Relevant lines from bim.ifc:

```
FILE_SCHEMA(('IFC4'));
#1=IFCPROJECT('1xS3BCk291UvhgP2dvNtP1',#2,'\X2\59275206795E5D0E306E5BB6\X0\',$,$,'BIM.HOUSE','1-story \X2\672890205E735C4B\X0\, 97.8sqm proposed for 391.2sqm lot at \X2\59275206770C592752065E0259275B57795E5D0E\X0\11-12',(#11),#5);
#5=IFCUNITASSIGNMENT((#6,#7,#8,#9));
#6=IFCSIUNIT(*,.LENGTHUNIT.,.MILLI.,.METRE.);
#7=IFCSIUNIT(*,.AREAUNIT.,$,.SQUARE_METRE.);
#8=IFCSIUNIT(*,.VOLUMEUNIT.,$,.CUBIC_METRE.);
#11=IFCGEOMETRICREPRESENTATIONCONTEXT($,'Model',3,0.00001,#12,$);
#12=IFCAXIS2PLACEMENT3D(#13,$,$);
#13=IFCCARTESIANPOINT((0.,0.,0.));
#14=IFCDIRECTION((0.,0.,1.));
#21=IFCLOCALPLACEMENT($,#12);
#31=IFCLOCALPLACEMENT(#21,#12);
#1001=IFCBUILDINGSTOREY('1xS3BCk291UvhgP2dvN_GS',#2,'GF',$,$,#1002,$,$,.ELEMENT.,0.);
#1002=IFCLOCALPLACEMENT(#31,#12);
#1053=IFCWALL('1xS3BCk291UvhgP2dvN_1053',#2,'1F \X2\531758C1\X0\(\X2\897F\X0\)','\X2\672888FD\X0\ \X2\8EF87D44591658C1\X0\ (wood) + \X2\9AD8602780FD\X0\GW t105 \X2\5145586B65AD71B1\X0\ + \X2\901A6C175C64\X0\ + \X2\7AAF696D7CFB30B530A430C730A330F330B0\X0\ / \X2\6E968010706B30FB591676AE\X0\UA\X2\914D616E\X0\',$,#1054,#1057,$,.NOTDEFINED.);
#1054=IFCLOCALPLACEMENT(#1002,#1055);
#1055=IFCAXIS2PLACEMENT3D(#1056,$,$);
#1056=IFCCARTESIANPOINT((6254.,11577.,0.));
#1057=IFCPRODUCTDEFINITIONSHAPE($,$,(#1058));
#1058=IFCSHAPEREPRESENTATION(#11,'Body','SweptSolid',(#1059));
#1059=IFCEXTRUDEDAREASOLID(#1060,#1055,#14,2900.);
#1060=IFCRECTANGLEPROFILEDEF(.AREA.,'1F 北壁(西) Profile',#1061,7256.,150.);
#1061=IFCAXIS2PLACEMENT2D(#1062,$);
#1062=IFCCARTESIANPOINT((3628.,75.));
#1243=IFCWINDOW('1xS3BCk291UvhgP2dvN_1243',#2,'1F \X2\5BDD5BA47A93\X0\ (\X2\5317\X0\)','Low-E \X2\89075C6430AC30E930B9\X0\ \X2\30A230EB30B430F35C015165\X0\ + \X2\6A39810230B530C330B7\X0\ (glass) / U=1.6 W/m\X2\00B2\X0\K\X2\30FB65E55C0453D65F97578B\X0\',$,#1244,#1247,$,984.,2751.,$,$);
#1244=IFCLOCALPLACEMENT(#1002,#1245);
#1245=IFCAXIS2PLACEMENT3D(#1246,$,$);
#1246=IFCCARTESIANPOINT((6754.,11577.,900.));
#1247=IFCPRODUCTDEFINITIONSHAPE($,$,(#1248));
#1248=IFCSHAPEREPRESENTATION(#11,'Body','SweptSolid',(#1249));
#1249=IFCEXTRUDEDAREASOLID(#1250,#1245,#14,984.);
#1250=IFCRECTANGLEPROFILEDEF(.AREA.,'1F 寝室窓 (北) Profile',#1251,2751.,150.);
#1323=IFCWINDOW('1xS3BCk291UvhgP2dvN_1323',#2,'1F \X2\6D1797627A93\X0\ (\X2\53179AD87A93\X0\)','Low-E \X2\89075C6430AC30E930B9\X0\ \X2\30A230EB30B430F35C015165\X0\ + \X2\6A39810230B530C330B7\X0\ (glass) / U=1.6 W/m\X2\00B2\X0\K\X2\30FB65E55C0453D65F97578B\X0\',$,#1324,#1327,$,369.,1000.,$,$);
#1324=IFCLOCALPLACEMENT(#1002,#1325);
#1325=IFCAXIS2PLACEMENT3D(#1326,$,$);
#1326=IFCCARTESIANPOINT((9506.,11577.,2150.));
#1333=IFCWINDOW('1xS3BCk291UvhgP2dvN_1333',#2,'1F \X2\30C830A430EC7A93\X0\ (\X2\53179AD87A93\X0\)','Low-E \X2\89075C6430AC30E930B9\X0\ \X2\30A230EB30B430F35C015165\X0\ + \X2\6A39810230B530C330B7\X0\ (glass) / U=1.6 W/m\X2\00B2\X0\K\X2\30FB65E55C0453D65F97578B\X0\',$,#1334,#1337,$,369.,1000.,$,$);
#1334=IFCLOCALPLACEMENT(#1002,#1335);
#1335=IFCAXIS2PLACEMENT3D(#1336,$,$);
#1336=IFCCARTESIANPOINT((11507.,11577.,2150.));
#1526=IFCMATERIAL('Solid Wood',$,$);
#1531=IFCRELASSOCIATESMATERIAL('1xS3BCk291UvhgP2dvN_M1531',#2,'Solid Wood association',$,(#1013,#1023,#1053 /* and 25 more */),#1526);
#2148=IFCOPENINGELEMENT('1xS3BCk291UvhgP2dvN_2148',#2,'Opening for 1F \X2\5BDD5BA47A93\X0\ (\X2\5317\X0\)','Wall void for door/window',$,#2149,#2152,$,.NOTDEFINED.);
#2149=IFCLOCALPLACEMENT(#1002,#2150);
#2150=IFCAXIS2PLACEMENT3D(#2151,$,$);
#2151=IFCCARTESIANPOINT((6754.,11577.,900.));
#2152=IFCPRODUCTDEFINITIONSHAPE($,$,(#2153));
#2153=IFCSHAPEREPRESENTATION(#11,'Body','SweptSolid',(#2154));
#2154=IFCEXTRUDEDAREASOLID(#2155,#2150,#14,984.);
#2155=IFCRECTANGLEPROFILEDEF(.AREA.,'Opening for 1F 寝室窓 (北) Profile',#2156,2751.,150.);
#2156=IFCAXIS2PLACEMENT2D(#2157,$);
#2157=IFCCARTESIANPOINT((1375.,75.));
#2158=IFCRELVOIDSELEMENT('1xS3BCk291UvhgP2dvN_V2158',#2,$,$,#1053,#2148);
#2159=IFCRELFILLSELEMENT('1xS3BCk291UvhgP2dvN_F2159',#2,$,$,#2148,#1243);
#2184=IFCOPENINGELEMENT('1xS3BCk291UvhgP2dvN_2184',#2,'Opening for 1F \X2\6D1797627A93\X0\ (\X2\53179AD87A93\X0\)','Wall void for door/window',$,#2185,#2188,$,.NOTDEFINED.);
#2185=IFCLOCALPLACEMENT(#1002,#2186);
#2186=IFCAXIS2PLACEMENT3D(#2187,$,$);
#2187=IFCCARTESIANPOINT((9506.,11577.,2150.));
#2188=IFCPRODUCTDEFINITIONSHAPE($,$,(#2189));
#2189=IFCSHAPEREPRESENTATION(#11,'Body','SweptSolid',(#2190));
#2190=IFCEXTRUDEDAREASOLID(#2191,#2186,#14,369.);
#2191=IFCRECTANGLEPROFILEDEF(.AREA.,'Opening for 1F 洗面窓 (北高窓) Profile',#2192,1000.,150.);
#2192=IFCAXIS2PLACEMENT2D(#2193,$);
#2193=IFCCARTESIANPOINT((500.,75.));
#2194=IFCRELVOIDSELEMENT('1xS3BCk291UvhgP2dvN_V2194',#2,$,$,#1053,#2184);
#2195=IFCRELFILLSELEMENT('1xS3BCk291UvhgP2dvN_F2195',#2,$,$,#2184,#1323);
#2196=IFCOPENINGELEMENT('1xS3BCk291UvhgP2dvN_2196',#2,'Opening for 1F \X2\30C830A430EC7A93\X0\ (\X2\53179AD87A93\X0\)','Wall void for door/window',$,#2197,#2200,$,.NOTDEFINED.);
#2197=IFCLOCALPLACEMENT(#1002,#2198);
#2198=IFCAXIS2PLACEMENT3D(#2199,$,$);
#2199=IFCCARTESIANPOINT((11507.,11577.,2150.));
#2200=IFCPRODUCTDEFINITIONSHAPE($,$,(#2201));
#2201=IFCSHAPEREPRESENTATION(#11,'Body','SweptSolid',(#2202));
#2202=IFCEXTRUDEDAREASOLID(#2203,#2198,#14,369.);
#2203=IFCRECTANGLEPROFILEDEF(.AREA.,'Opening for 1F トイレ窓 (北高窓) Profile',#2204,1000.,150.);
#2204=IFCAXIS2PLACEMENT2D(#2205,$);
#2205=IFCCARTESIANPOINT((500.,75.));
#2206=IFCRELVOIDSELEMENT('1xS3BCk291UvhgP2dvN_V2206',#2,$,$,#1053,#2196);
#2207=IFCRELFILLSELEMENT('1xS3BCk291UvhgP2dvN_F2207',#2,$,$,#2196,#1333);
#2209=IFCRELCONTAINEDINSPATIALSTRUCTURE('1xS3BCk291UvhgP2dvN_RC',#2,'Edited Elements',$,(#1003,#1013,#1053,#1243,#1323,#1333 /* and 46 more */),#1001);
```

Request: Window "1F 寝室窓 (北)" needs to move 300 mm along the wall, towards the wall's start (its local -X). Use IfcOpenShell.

```python
import ifcopenshell
import ifcopenshell.api.geometry
import ifcopenshell.util.placement

model = ifcopenshell.open("bim.ifc")

window = model.by_guid("1xS3BCk291UvhgP2dvN_1243")
opening = window.FillsVoids[0].RelatingOpeningElement
wall = opening.VoidsElements[0].RelatingBuildingElement

wall_matrix = ifcopenshell.util.placement.get_local_placement(wall.ObjectPlacement)
shift = wall_matrix[:3, 0] * -300.0
before = ifcopenshell.util.placement.get_local_placement(window.ObjectPlacement)[:3, 3].copy()

# The window is not placed relative to its opening, so move both.
for product in (opening, window):
    matrix = ifcopenshell.util.placement.get_local_placement(product.ObjectPlacement)
    matrix[:3, 3] += shift
    ifcopenshell.api.geometry.edit_object_placement(model, product=product, matrix=matrix, is_si=False)

after = ifcopenshell.util.placement.get_local_placement(window.ObjectPlacement)[:3, 3]
print("window moved by", (after - before).round(3) + 0.0)

model.write("bim_v2.ifc")
```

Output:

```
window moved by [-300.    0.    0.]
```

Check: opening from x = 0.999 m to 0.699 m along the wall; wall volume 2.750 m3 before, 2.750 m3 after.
